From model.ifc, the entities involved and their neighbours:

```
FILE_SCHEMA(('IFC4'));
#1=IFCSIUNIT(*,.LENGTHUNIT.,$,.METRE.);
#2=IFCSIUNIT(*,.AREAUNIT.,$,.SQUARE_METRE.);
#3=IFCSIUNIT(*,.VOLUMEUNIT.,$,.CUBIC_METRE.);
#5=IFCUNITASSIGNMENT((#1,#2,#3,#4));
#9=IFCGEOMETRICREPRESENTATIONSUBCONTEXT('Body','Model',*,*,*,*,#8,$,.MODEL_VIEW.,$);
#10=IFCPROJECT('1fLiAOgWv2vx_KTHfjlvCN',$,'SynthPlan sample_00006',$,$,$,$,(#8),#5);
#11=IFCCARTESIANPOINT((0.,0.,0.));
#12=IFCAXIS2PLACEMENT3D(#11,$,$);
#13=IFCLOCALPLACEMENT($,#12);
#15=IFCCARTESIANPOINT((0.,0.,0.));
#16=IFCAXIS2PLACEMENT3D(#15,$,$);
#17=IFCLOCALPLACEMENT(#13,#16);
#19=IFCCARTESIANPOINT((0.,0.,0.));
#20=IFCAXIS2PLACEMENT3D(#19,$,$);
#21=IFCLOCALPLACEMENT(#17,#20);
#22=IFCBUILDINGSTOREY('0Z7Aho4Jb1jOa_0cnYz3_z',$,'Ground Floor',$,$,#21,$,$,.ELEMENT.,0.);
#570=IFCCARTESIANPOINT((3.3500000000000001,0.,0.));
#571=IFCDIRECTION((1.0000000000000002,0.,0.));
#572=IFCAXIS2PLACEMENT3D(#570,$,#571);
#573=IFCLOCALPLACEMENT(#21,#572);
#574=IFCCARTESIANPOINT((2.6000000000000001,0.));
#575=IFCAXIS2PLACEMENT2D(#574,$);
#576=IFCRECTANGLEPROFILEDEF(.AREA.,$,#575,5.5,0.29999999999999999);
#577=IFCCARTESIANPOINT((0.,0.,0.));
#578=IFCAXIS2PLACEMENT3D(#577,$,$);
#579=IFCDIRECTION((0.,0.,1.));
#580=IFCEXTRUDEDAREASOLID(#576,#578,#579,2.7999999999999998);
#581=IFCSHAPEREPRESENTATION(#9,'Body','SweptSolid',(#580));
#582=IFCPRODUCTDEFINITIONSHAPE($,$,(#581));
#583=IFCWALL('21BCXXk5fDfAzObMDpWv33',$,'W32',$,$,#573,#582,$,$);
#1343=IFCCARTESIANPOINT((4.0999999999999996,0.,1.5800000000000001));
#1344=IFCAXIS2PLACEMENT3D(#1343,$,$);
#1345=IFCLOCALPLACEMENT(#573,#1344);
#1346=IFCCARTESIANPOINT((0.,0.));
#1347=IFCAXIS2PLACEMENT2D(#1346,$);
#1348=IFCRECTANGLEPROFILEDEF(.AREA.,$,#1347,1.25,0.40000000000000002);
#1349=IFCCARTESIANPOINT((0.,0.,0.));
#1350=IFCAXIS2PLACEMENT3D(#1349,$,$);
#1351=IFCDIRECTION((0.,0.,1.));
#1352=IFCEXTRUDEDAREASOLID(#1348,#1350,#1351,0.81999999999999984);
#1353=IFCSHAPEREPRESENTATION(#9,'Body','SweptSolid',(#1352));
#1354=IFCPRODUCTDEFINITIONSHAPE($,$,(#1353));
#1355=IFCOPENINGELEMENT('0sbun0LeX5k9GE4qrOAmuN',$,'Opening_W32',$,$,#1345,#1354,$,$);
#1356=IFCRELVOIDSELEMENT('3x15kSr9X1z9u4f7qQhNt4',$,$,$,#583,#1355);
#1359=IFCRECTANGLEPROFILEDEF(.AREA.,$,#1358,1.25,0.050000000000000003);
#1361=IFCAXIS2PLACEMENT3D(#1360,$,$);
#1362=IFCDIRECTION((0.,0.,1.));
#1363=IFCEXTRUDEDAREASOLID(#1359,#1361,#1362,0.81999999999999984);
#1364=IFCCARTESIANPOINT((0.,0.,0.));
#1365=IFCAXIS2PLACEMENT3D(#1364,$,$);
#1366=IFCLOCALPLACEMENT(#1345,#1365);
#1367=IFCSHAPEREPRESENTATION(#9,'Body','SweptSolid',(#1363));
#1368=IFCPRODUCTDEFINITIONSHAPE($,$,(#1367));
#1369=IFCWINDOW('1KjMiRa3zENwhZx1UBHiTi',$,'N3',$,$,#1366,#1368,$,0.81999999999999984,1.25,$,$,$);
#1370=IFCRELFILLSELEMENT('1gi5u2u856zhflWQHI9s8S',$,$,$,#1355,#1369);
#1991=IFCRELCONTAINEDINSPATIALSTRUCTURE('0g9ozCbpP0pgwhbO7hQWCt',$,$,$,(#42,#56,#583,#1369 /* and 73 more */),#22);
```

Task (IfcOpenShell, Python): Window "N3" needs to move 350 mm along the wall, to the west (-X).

```python
import ifcopenshell
import ifcopenshell.api.geometry
import ifcopenshell.util.placement

model = ifcopenshell.open("model.ifc")

window = model.by_guid("1KjMiRa3zENwhZx1UBHiTi")
opening = window.FillsVoids[0].RelatingOpeningElement
wall = opening.VoidsElements[0].RelatingBuildingElement

wall_matrix = ifcopenshell.util.placement.get_local_placement(wall.ObjectPlacement)
shift = wall_matrix[:3, 0] * -0.35
before = ifcopenshell.util.placement.get_local_placement(window.ObjectPlacement)[:3, 3].copy()

# The window is placed relative to its opening, so it follows when the opening moves.
matrix = ifcopenshell.util.placement.get_local_placement(opening.ObjectPlacement)
matrix[:3, 3] += shift
ifcopenshell.api.geometry.edit_object_placement(
    model, product=opening, matrix=matrix, is_si=False, should_transform_children=True
)

after = ifcopenshell.util.placement.get_local_placement(window.ObjectPlacement)[:3, 3]
print("window moved by", (after - before).round(3) + 0.0)

model.write("model_updated.ifc")
```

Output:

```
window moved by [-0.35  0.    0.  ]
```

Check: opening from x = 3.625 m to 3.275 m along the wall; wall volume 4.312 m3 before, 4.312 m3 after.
